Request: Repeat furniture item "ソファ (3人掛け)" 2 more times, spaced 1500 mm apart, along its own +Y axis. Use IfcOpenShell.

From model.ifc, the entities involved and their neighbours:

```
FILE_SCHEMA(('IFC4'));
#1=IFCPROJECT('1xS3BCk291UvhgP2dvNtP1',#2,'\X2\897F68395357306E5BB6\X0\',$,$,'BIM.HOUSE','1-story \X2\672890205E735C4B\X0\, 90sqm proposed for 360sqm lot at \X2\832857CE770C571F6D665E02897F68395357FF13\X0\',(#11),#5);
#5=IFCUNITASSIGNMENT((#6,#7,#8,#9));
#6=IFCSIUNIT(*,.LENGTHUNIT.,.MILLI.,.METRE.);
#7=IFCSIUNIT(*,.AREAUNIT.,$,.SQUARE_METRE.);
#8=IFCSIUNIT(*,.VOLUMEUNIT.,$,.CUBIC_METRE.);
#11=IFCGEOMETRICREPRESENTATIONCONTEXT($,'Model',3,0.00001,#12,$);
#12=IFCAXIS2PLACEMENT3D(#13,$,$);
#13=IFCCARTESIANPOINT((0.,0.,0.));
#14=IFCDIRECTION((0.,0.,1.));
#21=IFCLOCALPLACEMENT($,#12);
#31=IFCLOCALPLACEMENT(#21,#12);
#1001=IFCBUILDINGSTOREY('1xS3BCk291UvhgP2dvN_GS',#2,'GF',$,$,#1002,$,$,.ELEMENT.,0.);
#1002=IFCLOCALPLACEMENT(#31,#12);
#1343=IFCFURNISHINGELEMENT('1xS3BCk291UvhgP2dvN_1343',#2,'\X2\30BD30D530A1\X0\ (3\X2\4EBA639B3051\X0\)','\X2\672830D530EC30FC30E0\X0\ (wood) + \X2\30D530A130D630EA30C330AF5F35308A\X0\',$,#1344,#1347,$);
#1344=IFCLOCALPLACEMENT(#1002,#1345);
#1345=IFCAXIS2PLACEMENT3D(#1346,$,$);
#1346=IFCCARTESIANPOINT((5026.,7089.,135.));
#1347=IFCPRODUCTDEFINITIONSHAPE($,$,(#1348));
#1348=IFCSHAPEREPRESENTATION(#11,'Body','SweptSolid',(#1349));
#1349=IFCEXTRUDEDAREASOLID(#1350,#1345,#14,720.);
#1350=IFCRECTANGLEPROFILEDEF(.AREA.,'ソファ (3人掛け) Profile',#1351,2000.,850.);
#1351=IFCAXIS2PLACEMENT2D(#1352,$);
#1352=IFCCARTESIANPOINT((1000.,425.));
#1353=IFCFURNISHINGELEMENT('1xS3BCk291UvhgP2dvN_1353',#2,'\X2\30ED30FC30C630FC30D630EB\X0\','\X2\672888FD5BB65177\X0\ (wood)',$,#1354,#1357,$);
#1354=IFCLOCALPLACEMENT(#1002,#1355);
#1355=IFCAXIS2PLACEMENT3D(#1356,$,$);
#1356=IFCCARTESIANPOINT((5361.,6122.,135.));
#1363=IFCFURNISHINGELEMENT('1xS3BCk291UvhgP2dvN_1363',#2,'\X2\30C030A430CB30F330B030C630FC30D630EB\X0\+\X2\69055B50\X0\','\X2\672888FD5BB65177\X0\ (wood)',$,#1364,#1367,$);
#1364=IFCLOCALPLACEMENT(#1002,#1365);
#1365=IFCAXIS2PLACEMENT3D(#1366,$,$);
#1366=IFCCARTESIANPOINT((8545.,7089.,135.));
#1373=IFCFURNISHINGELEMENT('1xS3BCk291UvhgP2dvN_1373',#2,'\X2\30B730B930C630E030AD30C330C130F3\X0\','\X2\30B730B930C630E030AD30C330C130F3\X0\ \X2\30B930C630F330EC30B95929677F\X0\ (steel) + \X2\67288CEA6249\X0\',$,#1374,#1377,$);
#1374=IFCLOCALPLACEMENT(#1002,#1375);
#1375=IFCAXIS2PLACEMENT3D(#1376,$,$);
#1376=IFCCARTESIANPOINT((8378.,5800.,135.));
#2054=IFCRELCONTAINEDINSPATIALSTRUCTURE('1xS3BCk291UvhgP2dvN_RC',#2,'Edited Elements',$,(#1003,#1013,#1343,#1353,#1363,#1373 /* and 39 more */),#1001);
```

```python
import ifcopenshell
import ifcopenshell.api.geometry
import ifcopenshell.api.root
import ifcopenshell.util.element
import ifcopenshell.util.placement
import ifcopenshell.util.unit

model = ifcopenshell.open("model.ifc")
unit_scale = ifcopenshell.util.unit.calculate_unit_scale(model)


def reuse_history(source, copy):
    """copy_class also copies each property set's owner history, people and application; keep the originals."""
    for rel in copy.IsDefinedBy:
        if rel.is_a("IfcRelDefinesByProperties") and (history := rel.RelatingPropertyDefinition.OwnerHistory):
            rel.RelatingPropertyDefinition.OwnerHistory = source.OwnerHistory
            ifcopenshell.util.element.remove_deep2(model, history)


source = model.by_guid("1xS3BCk291UvhgP2dvN_1343")
base = ifcopenshell.util.placement.get_local_placement(source.ObjectPlacement)
step = base[:3, 1] * 1.5 / unit_scale

for i in range(1, 3):
    copy = ifcopenshell.api.root.copy_class(model, product=source)
    copy.Representation = ifcopenshell.util.element.copy_deep(
        model, source.Representation, exclude=["IfcGeometricRepresentationContext", "IfcRepresentationMap"]
    )
    reuse_history(source, copy)
    matrix = base.copy()
    matrix[:3, 3] += i * step
    print("added at", matrix[:3, 3].round(3) + 0.0)
    ifcopenshell.api.geometry.edit_object_placement(model, product=copy, matrix=matrix, is_si=False)

model.write("model_edited.ifc")
```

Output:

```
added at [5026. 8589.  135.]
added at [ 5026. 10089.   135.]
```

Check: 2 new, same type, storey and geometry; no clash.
